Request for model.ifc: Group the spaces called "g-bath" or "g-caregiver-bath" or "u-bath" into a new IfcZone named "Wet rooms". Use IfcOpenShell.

First a look at what the model holds.

```python
import ifcopenshell

model = ifcopenshell.open("model.ifc")
print(model.schema)
seen = {}
for space in model.by_type("IfcSpace"):
    seen[space.LongName] = seen.get(space.LongName, 0) + 1
for name, count in sorted(seen.items(), key=str):
    print(count, "x", name)
print("zones:", [z.Name for z in model.by_type("IfcZone")][:20])
```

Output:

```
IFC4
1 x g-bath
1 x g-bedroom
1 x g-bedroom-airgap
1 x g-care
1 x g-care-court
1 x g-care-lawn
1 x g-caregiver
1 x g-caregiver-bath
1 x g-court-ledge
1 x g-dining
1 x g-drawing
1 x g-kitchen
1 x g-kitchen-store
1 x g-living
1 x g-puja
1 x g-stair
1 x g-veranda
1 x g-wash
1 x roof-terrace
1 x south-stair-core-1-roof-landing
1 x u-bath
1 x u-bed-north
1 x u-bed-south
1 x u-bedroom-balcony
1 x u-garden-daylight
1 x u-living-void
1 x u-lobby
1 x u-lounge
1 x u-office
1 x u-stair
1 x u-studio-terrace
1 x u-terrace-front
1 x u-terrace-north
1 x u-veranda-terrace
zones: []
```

```python
import ifcopenshell
import ifcopenshell.api.group
import ifcopenshell.api.root

model = ifcopenshell.open("model.ifc")

names = {"g-bath", "g-caregiver-bath", "u-bath"}
spaces = [s for s in model.by_type("IfcSpace") if s.LongName in names]

zone = ifcopenshell.api.root.create_entity(model, ifc_class="IfcZone", name="Wet rooms")
ifcopenshell.api.group.assign_group(model, products=spaces, group=zone)
print(len(spaces), "spaces in", zone.Name)

model.write("model_v2.ifc")
```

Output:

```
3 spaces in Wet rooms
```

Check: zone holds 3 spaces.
